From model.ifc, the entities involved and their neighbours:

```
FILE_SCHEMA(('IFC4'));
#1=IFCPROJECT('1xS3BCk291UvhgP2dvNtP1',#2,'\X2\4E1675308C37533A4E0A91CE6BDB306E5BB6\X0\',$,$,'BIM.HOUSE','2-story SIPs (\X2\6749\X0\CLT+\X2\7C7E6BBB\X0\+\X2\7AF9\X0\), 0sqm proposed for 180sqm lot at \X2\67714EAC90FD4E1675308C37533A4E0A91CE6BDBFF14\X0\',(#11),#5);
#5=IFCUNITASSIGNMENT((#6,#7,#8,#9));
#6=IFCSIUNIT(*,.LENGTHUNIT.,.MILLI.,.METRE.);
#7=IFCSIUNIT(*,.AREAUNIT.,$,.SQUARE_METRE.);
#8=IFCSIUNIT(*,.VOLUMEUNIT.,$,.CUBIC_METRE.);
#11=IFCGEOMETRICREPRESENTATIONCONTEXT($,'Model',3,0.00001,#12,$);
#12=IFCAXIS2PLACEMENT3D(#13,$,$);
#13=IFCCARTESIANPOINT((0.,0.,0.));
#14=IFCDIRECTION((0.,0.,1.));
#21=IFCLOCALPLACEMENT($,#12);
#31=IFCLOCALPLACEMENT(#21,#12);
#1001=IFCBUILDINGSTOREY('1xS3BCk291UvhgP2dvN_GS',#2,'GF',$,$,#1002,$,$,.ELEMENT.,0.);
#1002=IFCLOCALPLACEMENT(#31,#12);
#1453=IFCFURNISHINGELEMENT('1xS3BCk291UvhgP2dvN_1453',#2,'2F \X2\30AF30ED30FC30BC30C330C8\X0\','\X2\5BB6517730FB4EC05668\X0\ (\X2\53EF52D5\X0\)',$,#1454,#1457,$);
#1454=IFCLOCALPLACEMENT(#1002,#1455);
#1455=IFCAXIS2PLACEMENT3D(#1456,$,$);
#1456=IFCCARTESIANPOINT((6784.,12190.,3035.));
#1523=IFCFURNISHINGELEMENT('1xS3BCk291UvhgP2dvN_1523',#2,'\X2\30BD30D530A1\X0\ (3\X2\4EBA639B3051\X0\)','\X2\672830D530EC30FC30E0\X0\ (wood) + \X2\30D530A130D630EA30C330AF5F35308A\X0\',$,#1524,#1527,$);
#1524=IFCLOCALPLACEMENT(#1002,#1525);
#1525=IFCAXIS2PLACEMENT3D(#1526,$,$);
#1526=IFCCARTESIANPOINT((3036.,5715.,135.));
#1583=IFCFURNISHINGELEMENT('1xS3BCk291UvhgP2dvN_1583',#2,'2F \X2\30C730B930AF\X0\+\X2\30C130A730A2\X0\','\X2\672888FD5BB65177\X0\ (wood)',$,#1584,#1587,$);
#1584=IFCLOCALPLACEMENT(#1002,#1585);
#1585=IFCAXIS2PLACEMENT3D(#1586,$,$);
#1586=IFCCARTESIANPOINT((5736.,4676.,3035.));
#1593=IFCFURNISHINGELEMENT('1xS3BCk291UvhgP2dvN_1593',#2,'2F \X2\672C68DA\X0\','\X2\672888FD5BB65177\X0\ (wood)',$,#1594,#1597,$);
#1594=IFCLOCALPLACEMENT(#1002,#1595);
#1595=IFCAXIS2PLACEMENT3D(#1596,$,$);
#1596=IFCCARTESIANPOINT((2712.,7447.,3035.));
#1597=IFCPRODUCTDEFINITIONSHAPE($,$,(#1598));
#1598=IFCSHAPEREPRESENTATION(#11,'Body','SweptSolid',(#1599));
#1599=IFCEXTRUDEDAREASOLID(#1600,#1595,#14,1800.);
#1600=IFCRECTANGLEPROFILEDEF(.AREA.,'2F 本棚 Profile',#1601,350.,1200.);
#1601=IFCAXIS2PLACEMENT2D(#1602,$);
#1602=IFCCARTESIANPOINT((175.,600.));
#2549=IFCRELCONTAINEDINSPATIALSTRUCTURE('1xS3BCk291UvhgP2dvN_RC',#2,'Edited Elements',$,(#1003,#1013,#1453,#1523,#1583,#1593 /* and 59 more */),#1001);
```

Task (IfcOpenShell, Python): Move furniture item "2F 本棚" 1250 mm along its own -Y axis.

```python
import ifcopenshell
import ifcopenshell.api.geometry
import ifcopenshell.util.placement

model = ifcopenshell.open("model.ifc")

item = model.by_guid("1xS3BCk291UvhgP2dvN_1593")
matrix = ifcopenshell.util.placement.get_local_placement(item.ObjectPlacement)
matrix[:3, 3] -= matrix[:3, 1] * 1250.0
ifcopenshell.api.geometry.edit_object_placement(model, product=item, matrix=matrix, is_si=False)

print(ifcopenshell.util.placement.get_local_placement(item.ObjectPlacement).round(3) + 0.0)

model.write("model_edited.ifc")
```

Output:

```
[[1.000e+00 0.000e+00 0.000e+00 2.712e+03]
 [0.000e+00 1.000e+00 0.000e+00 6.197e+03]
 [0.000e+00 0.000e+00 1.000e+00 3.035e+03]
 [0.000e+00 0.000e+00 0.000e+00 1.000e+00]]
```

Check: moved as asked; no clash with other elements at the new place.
